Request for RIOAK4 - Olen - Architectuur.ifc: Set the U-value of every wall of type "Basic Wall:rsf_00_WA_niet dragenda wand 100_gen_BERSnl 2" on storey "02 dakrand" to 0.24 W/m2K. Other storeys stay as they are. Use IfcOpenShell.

First a look at what the model holds.

```python
import ifcopenshell
import ifcopenshell.util.element

model = ifcopenshell.open("RIOAK4 - Olen - Architectuur.ifc")
print(model.schema)
storey = next(s for s in model.by_type("IfcBuildingStorey") if s.Name == "02 dakrand")
walls = [e for e in ifcopenshell.util.element.get_decomposition(storey) if e.is_a("IfcWall")]
seen = {}
for e in walls:
    element_type = ifcopenshell.util.element.get_type(e)
    key = (element_type.Name if element_type != e and element_type else None, ifcopenshell.util.element.get_pset(e, "Pset_WallCommon", "ThermalTransmittance"))
    seen[key] = seen.get(key, 0) + 1
for (name, value), count in sorted(seen.items(), key=str):
    print(count, "x", name, "|", value)
```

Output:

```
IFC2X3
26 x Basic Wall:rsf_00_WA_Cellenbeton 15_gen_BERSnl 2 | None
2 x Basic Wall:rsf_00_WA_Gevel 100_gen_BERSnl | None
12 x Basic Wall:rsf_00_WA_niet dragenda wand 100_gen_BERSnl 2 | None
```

```python
import ifcopenshell
import ifcopenshell.api.pset
import ifcopenshell.util.element

model = ifcopenshell.open("RIOAK4 - Olen - Architectuur.ifc")

storey = next(s for s in model.by_type("IfcBuildingStorey") if s.Name == "02 dakrand")
walls = [e for e in ifcopenshell.util.element.get_decomposition(storey) if e.is_a("IfcWall")]

count = 0
for e in walls:
    element_type = ifcopenshell.util.element.get_type(e)
    if element_type in (None, e) or element_type.Name != "Basic Wall:rsf_00_WA_niet dragenda wand 100_gen_BERSnl 2":
        continue
    # add_pset returns the element's existing set when there is one.
    pset = ifcopenshell.api.pset.add_pset(model, product=e, name="Pset_WallCommon")
    ifcopenshell.api.pset.edit_pset(model, pset=pset, properties={"ThermalTransmittance": 0.24})
    count += 1

print(count, "walls updated")

model.write("RIOAK4 - Olen - Architectuur_v2.ifc")
```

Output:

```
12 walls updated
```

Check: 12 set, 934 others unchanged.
